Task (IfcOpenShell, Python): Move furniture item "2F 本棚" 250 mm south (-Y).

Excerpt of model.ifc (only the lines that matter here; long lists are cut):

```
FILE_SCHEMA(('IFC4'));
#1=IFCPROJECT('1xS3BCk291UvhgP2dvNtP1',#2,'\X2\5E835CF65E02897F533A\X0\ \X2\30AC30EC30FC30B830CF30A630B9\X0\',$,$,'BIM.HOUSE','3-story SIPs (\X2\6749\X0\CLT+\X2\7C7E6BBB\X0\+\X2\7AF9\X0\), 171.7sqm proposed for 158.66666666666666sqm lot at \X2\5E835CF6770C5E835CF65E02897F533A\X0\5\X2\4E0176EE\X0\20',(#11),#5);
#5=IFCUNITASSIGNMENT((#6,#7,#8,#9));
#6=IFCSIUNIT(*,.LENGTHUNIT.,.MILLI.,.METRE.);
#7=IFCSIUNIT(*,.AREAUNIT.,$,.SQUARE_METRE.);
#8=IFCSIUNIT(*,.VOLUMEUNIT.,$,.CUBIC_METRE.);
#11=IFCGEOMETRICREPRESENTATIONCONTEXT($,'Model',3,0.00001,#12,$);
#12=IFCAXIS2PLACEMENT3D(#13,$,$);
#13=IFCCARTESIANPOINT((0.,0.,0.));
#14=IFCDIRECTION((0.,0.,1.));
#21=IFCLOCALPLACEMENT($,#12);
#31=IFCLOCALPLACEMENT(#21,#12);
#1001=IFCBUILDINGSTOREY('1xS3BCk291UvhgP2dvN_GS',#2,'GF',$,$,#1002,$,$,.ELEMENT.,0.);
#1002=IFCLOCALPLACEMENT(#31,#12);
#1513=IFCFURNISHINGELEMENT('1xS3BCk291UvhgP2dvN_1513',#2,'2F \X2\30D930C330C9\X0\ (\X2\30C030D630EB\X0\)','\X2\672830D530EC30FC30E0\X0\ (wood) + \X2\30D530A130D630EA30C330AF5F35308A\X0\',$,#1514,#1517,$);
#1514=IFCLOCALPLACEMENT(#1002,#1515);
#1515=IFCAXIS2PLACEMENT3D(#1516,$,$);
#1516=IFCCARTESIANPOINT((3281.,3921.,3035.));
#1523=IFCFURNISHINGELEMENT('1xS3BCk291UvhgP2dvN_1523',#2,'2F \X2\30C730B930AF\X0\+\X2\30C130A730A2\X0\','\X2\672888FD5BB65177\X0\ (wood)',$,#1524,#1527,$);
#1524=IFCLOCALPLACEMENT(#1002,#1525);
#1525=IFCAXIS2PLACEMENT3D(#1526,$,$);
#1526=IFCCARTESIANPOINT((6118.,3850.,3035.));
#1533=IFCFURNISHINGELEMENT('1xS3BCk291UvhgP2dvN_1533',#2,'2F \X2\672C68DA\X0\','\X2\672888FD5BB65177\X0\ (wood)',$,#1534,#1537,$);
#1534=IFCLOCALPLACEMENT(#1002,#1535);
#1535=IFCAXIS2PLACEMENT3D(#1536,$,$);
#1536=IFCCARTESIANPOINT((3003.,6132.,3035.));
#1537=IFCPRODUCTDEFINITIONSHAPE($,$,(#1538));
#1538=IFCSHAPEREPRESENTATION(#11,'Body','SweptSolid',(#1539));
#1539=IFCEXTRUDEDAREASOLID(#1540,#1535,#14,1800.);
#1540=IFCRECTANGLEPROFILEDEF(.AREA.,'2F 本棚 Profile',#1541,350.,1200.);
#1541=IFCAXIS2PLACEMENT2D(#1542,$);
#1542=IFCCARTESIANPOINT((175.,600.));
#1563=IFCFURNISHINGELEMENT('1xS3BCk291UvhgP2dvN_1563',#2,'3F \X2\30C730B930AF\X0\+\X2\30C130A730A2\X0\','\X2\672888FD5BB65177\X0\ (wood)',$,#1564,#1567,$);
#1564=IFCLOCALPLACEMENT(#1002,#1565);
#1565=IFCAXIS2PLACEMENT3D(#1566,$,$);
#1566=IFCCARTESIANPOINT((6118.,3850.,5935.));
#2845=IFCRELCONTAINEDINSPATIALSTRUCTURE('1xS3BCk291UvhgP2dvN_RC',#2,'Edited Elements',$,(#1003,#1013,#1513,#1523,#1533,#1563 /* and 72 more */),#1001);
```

```python
import ifcopenshell
import ifcopenshell.api.geometry
import ifcopenshell.util.placement
import ifcopenshell.util.unit

model = ifcopenshell.open("model.ifc")
unit_scale = ifcopenshell.util.unit.calculate_unit_scale(model)

item = model.by_guid("1xS3BCk291UvhgP2dvN_1533")
matrix = ifcopenshell.util.placement.get_local_placement(item.ObjectPlacement)
matrix[1, 3] -= 0.25 / unit_scale
ifcopenshell.api.geometry.edit_object_placement(model, product=item, matrix=matrix, is_si=False)

print(ifcopenshell.util.placement.get_local_placement(item.ObjectPlacement).round(3) + 0.0)

model.write("model_rev.ifc")
```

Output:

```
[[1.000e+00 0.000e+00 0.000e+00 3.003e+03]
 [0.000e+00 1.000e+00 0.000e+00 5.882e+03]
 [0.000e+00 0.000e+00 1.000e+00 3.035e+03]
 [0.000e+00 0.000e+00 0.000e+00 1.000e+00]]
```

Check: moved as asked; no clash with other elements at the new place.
